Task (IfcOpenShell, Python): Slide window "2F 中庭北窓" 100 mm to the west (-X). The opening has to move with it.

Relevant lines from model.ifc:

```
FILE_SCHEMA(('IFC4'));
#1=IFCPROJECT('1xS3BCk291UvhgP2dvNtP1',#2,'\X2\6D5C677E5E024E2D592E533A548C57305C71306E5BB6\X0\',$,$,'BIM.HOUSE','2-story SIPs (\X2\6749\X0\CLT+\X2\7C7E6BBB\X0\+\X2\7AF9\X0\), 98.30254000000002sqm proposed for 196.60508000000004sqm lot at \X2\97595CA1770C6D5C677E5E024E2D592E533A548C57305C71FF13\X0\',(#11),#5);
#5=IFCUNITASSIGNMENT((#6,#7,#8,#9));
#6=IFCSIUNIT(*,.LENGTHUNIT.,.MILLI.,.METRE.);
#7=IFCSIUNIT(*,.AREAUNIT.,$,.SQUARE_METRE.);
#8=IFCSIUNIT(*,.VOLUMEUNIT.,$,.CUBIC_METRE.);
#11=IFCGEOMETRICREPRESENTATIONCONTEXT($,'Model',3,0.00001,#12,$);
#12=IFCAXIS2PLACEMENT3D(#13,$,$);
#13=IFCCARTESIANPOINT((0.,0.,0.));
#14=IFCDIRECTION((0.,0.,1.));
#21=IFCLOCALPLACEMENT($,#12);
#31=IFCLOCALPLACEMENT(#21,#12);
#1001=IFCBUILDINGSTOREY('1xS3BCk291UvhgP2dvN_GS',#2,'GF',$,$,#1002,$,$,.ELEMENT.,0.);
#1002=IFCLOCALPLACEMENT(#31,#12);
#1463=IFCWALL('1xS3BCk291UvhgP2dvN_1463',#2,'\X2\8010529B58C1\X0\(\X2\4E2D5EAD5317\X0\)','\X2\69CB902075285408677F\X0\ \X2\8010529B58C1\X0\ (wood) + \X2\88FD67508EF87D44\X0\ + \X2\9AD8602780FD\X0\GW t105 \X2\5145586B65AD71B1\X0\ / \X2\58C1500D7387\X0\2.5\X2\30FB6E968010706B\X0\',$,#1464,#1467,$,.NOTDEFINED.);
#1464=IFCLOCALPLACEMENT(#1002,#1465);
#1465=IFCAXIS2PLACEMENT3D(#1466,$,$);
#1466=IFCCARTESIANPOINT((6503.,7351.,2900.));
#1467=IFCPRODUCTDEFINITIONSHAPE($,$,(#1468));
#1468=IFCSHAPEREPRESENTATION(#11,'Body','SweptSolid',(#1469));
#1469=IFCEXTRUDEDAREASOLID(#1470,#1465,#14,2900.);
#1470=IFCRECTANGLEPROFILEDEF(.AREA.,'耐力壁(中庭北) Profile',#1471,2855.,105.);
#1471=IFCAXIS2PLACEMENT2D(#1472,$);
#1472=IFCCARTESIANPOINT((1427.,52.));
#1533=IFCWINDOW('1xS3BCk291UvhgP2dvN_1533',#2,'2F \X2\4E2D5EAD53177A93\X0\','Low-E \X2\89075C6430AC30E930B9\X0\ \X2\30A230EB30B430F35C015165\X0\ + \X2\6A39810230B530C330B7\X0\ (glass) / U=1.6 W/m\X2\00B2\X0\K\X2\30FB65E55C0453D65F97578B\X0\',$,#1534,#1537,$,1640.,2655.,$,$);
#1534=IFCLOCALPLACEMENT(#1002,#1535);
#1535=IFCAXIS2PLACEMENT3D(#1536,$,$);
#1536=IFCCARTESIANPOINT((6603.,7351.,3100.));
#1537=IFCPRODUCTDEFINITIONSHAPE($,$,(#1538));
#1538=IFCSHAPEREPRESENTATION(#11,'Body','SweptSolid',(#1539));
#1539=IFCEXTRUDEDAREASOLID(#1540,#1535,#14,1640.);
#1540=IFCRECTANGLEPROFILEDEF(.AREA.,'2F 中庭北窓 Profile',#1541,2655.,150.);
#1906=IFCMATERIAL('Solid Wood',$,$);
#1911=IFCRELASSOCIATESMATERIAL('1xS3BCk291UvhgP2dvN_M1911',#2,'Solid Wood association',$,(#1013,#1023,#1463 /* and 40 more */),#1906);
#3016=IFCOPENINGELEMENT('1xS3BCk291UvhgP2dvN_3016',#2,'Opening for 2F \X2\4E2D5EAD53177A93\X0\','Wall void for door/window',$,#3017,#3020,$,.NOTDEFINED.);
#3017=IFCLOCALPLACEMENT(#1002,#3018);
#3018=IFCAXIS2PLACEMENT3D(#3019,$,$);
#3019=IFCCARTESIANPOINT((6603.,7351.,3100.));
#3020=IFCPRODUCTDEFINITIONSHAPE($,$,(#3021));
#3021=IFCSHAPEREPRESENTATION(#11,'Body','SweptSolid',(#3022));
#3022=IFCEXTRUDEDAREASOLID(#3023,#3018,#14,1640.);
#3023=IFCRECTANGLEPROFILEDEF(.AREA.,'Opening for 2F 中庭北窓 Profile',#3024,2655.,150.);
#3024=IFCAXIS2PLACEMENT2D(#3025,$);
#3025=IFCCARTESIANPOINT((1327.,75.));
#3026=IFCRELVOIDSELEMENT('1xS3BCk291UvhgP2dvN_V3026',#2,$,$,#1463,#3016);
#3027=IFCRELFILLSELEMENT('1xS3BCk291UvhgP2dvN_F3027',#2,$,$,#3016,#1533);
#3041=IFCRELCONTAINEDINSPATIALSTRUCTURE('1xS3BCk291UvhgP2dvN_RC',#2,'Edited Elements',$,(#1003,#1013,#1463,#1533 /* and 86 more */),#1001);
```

```python
import ifcopenshell
import ifcopenshell.api.geometry
import ifcopenshell.util.placement

model = ifcopenshell.open("model.ifc")

window = model.by_guid("1xS3BCk291UvhgP2dvN_1533")
opening = window.FillsVoids[0].RelatingOpeningElement
wall = opening.VoidsElements[0].RelatingBuildingElement

wall_matrix = ifcopenshell.util.placement.get_local_placement(wall.ObjectPlacement)
shift = wall_matrix[:3, 0] * -100.0
before = ifcopenshell.util.placement.get_local_placement(window.ObjectPlacement)[:3, 3].copy()

# The window is not placed relative to its opening, so move both.
for product in (opening, window):
    matrix = ifcopenshell.util.placement.get_local_placement(product.ObjectPlacement)
    matrix[:3, 3] += shift
    ifcopenshell.api.geometry.edit_object_placement(model, product=product, matrix=matrix, is_si=False)

after = ifcopenshell.util.placement.get_local_placement(window.ObjectPlacement)[:3, 3]
print("window moved by", (after - before).round(3) + 0.0)

model.write("model_updated.ifc")
```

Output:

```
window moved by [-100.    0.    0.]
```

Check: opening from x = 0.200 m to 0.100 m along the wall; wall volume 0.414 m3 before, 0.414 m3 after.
